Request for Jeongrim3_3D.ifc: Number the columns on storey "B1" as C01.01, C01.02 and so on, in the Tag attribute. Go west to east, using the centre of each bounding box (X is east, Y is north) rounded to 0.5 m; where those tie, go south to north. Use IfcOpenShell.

First a look at what the model holds.

```python
import ifcopenshell
import ifcopenshell.util.element
import ifcopenshell.util.placement

model = ifcopenshell.open("Jeongrim3_3D.ifc")
print(model.schema)
storey = next(s for s in model.by_type("IfcBuildingStorey") if s.Name == "B1")
columns = [e for e in ifcopenshell.util.element.get_decomposition(storey) if e.is_a("IfcColumn")]
for e in sorted(columns, key=lambda e: e.id()):
    origin = ifcopenshell.util.placement.get_local_placement(e.ObjectPlacement)[:3, 3]
    print(e.id(), e.Tag, e.Name, origin.round(2) + 0.0, sep=" | ")
```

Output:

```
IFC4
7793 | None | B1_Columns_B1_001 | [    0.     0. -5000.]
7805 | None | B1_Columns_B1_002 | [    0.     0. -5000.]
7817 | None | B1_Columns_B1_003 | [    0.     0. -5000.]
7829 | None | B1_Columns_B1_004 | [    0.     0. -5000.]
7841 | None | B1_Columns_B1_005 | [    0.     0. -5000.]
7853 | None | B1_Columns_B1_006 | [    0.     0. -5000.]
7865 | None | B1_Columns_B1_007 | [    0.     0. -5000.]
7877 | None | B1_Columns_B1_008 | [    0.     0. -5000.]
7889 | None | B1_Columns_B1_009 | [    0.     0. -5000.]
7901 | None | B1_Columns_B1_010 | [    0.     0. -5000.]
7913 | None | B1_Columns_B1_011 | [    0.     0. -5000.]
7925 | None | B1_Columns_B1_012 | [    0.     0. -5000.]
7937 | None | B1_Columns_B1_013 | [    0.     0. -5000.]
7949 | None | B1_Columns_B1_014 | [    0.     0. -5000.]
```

```python
import ifcopenshell
import ifcopenshell.geom
import ifcopenshell.util.element
import ifcopenshell.util.shape

model = ifcopenshell.open("Jeongrim3_3D.ifc")
settings = ifcopenshell.geom.settings()
settings.set("use-world-coords", True)


def centre(element):
    shape = ifcopenshell.geom.create_shape(settings, element)
    return ifcopenshell.util.shape.get_bbox_centroid(shape.geometry)


storey = next(s for s in model.by_type("IfcBuildingStorey") if s.Name == "B1")
columns = [e for e in ifcopenshell.util.element.get_decomposition(storey) if e.is_a("IfcColumn")]

# Insertion points can sit at a corner or the storey origin, so sort by the geometry (in metres).
centres = {e: centre(e) for e in columns}
columns.sort(key=lambda e: (round(centres[e][0] / 0.5), centres[e][1]))

for i, e in enumerate(columns, start=1):
    number = f"C01.{i:02d}"
    e.Tag = number
    print(e.id(), number)

model.write("Jeongrim3_3D_edited.ifc")
```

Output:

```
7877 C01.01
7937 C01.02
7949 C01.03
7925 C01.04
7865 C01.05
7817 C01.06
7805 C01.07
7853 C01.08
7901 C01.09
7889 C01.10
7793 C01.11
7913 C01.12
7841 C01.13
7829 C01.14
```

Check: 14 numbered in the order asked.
